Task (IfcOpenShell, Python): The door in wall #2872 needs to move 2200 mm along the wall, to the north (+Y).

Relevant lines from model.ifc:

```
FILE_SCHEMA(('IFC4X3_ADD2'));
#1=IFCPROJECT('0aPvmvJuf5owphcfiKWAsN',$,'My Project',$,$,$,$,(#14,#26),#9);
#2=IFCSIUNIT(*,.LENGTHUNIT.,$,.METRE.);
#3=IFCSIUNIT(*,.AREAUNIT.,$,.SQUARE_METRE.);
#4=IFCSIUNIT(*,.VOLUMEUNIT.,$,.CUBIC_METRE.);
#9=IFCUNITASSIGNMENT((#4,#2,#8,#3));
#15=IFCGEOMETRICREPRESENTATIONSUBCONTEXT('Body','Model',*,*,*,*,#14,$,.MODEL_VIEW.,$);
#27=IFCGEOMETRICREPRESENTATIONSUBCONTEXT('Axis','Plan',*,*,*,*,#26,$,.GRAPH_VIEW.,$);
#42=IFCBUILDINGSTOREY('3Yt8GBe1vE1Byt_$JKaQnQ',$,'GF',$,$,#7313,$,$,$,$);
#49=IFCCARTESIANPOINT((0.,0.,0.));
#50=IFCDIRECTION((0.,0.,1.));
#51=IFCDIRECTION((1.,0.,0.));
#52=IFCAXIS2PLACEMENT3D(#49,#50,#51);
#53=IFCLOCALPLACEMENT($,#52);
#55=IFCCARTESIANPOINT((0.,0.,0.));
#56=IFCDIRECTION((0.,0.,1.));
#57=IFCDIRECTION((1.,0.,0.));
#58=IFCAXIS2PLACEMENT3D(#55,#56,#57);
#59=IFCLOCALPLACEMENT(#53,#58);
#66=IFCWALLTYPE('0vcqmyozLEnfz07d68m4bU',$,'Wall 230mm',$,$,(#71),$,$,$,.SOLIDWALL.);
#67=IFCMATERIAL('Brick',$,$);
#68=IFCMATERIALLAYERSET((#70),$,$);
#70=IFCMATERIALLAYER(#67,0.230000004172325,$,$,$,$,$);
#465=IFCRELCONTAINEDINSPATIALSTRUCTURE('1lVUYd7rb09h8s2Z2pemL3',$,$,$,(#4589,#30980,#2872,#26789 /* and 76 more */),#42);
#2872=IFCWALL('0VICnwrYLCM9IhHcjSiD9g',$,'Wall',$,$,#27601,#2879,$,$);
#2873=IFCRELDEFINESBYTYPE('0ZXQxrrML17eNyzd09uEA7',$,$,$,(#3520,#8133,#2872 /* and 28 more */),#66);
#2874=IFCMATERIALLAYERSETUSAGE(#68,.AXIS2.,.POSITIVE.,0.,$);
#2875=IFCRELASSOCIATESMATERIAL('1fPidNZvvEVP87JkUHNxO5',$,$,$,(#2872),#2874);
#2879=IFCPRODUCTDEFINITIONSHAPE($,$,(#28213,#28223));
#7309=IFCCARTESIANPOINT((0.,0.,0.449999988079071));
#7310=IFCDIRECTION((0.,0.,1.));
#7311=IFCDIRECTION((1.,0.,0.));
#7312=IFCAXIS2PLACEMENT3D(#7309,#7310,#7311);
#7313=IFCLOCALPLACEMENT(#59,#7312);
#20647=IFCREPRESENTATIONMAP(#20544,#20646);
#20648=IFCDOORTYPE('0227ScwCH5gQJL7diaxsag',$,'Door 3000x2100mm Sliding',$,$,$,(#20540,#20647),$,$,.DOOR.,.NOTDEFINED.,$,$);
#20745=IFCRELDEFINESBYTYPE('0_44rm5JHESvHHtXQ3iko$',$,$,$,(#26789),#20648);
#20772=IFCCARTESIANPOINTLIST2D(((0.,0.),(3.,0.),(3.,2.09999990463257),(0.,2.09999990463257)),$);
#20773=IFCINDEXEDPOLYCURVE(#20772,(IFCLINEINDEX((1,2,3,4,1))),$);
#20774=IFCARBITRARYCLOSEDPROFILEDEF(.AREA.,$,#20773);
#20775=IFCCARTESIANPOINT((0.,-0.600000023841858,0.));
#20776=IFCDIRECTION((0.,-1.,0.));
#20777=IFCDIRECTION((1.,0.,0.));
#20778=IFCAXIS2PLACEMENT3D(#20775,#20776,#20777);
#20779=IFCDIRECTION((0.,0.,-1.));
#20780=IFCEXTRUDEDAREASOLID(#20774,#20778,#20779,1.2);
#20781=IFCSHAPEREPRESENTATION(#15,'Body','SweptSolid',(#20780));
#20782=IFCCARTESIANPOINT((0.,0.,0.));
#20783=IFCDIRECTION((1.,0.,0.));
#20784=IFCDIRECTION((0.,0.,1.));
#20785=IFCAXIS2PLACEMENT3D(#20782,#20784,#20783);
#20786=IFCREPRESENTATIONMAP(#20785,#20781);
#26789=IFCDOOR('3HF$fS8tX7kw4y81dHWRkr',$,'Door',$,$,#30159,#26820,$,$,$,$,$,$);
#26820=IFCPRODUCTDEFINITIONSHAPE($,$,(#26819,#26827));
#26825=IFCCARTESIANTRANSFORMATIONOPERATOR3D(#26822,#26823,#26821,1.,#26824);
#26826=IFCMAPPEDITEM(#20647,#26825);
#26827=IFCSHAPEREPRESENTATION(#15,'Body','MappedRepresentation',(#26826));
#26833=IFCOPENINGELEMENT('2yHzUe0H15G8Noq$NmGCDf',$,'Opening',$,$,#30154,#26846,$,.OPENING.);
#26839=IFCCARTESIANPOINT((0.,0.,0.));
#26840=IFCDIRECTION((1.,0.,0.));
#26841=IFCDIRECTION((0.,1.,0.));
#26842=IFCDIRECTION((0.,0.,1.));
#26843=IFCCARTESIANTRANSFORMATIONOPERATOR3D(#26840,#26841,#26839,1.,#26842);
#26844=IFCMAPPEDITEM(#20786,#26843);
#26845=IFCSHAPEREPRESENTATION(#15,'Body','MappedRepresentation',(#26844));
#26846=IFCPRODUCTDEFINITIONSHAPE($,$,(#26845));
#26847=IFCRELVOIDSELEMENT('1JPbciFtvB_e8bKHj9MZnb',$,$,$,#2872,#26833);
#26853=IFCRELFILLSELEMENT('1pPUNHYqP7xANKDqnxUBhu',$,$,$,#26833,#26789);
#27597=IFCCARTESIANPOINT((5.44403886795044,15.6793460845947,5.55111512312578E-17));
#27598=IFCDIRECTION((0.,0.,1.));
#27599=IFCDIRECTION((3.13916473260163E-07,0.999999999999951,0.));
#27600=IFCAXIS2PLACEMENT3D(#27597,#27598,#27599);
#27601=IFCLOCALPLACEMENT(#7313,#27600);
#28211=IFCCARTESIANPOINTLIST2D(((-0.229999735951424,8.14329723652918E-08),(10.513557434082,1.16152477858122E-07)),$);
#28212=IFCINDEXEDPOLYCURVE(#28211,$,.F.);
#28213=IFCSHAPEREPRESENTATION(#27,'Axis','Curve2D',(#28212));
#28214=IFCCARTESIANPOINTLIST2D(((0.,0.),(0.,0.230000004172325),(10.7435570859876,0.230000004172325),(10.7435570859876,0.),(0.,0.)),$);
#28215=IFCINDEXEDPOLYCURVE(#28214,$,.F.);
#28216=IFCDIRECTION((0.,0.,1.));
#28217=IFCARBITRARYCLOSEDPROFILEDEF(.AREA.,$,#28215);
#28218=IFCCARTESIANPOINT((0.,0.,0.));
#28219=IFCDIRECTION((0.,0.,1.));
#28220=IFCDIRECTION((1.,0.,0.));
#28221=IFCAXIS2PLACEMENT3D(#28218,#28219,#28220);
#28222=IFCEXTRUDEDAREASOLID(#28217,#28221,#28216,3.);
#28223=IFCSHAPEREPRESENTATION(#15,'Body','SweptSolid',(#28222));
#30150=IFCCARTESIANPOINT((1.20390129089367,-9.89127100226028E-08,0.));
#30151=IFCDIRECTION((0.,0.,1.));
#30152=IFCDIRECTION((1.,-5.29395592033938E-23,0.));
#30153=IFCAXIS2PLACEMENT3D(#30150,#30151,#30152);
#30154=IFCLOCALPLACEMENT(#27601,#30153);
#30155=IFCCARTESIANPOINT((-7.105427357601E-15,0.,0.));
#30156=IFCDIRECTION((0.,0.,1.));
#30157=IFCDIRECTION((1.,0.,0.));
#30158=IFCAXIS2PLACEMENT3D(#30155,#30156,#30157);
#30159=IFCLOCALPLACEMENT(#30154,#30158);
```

```python
import ifcopenshell
import ifcopenshell.api.geometry
import ifcopenshell.util.placement
import ifcopenshell.util.unit

model = ifcopenshell.open("model.ifc")
unit_scale = ifcopenshell.util.unit.calculate_unit_scale(model)

door = model.by_guid("3HF$fS8tX7kw4y81dHWRkr")
opening = door.FillsVoids[0].RelatingOpeningElement
wall = opening.VoidsElements[0].RelatingBuildingElement

wall_matrix = ifcopenshell.util.placement.get_local_placement(wall.ObjectPlacement)
shift = wall_matrix[:3, 0] * 2.2 / unit_scale
before = ifcopenshell.util.placement.get_local_placement(door.ObjectPlacement)[:3, 3].copy()

# The door is placed relative to its opening, so it follows when the opening moves.
matrix = ifcopenshell.util.placement.get_local_placement(opening.ObjectPlacement)
matrix[:3, 3] += shift
ifcopenshell.api.geometry.edit_object_placement(
    model, product=opening, matrix=matrix, is_si=False, should_transform_children=True
)

after = ifcopenshell.util.placement.get_local_placement(door.ObjectPlacement)[:3, 3]
print("door moved by", (after - before).round(3) + 0.0)

model.write("model_updated.ifc")
```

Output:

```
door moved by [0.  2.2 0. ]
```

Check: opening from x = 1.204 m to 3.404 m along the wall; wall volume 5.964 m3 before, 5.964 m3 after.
